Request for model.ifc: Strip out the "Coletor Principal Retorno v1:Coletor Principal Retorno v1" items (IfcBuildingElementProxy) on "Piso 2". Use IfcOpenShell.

First a look at what the model holds.

```python
import ifcopenshell
import ifcopenshell.util.element

model = ifcopenshell.open("model.ifc")
print(model.schema)
storey = next(s for s in model.by_type("IfcBuildingStorey") if s.Name == "Piso 2")
proxies = [e for e in ifcopenshell.util.element.get_decomposition(storey) if e.is_a("IfcBuildingElementProxy")]
seen = {}
for e in proxies:
    element_type = ifcopenshell.util.element.get_type(e)
    name = element_type.Name if element_type not in (None, e) else None
    seen[name] = seen.get(name, 0) + 1
for name, count in sorted(seen.items(), key=str):
    print(count, "x", name)
```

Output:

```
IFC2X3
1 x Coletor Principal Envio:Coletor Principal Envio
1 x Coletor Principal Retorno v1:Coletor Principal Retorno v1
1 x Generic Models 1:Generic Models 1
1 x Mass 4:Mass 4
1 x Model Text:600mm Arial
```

```python
import ifcopenshell
import ifcopenshell.api.root
import ifcopenshell.util.element

model = ifcopenshell.open("model.ifc")

storey = next(s for s in model.by_type("IfcBuildingStorey") if s.Name == "Piso 2")
proxies = [e for e in ifcopenshell.util.element.get_decomposition(storey) if e.is_a("IfcBuildingElementProxy")]
targets = [e for e in proxies if (t := ifcopenshell.util.element.get_type(e)) not in (None, e) and t.Name == "Coletor Principal Retorno v1:Coletor Principal Retorno v1"]

for e in targets:
    ifcopenshell.api.root.remove_product(model, product=e)
print(len(targets), "removed")

model.write("model_rev.ifc")
```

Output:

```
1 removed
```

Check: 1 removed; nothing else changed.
